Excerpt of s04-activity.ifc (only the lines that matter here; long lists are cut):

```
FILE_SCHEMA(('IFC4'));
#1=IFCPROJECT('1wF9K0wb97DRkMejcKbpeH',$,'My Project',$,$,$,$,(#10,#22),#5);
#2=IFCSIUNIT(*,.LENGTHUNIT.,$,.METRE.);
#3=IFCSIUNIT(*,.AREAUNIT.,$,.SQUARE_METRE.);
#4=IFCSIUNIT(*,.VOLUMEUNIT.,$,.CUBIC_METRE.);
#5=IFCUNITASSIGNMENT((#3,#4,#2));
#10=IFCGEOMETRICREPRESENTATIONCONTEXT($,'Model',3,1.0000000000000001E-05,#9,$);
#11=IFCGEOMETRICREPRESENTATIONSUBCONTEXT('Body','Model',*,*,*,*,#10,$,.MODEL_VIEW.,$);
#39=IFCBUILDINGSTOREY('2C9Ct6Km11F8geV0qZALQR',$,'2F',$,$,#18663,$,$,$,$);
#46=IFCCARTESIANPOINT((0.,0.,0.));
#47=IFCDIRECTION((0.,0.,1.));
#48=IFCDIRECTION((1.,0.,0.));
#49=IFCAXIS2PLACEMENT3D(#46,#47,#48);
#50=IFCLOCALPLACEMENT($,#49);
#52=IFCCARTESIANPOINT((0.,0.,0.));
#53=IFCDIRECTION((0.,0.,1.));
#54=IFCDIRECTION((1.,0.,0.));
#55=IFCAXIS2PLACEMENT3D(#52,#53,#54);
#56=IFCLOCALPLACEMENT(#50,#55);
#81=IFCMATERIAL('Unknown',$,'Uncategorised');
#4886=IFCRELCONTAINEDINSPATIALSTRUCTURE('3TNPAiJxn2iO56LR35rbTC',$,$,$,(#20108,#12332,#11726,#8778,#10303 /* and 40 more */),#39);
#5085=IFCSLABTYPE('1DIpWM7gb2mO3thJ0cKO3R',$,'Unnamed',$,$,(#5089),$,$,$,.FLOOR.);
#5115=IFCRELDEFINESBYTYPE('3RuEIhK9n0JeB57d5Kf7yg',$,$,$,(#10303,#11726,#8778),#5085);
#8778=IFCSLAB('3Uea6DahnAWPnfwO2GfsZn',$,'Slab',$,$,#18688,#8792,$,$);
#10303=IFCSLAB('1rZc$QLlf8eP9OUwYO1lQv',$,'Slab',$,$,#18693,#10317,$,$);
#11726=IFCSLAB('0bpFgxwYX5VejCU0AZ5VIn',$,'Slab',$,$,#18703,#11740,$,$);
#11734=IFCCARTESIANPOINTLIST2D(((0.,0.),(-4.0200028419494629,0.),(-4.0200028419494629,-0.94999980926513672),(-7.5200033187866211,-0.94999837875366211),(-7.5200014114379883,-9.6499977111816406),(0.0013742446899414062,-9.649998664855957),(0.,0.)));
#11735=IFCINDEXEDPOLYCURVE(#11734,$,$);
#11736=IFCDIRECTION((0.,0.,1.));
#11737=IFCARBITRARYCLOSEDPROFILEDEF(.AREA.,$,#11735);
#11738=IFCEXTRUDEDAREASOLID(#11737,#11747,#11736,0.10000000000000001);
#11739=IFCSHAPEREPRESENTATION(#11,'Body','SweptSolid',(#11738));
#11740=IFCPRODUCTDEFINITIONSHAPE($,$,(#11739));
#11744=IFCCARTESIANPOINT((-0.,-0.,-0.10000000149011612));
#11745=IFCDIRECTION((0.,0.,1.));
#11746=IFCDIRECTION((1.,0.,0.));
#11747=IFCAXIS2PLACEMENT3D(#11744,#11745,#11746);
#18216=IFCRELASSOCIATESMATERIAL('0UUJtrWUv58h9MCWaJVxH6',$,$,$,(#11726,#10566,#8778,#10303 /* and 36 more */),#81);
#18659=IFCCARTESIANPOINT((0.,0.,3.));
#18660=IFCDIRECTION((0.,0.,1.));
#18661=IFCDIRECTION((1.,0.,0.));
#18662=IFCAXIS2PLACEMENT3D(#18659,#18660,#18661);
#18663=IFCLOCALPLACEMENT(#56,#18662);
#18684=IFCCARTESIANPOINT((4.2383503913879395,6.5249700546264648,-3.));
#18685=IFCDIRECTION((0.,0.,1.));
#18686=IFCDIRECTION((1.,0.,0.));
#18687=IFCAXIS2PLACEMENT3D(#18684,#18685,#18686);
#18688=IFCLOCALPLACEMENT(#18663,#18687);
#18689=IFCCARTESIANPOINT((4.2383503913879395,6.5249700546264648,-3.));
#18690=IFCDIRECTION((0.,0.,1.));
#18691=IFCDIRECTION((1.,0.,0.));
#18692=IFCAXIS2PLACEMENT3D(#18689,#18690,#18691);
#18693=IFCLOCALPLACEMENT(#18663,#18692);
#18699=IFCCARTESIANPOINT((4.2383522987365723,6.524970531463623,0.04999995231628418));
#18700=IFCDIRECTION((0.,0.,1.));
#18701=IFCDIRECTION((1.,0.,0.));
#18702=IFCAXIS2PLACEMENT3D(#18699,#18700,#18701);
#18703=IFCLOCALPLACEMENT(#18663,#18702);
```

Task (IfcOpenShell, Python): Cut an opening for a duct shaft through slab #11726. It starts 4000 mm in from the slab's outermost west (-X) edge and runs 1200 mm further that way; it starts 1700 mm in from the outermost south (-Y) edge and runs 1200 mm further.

```python
import numpy as np
import ifcopenshell
import ifcopenshell.api.feature
import ifcopenshell.api.geometry
import ifcopenshell.api.root
import ifcopenshell.geom
import ifcopenshell.util.placement
import ifcopenshell.util.representation
import ifcopenshell.util.shape
import ifcopenshell.util.unit

model = ifcopenshell.open("s04-activity.ifc")
unit_scale = ifcopenshell.util.unit.calculate_unit_scale(model)
settings = ifcopenshell.geom.settings()


def volume(element):
    """Net volume in cubic metres, openings subtracted."""
    shape = ifcopenshell.geom.create_shape(settings, element)
    return ifcopenshell.util.shape.get_volume(shape.geometry)


slab = model.by_id(11726)
before = volume(slab)

# Extent in the slab's own axes, in metres. The edges named are its -X and -Y sides.
slab_shape = ifcopenshell.geom.create_shape(settings, slab)
vertices = ifcopenshell.util.shape.get_vertices(slab_shape.geometry)
x_min, y_min, bottom = vertices.min(axis=0)
top = vertices[:, 2].max()

opening = ifcopenshell.api.root.create_entity(model, ifc_class="IfcOpeningElement", name="Duct shaft opening", predefined_type="OPENING")
context = ifcopenshell.util.representation.get_context(model, "Model", "Body", "MODEL_VIEW")
width, depth = 1.2, 1.2
outline = [(0.0, 0.0), (width, 0.0), (width, depth), (0.0, depth), (0.0, 0.0)]
# Overshoot both faces by 50 mm so the cut is clean.
shape = ifcopenshell.api.geometry.add_slab_representation(
    model, context=context, depth=top - bottom + 0.1, polyline=outline
)
ifcopenshell.api.geometry.assign_representation(model, product=opening, representation=shape)

matrix = ifcopenshell.util.placement.get_local_placement(slab.ObjectPlacement)
matrix[:, 3] = matrix @ np.append(np.array([x_min + 4, y_min + 1.7, bottom - 0.05]) / unit_scale, 1.0)
ifcopenshell.api.geometry.edit_object_placement(model, product=opening, matrix=matrix, is_si=False)
ifcopenshell.api.feature.add_feature(model, feature=opening, element=slab)

after = volume(slab)

print(f"slab volume {before:.3f} -> {after:.3f} m3")

model.write("s04-activity_v2.ifc")
```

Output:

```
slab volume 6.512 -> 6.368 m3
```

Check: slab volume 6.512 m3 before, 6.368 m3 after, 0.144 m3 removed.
